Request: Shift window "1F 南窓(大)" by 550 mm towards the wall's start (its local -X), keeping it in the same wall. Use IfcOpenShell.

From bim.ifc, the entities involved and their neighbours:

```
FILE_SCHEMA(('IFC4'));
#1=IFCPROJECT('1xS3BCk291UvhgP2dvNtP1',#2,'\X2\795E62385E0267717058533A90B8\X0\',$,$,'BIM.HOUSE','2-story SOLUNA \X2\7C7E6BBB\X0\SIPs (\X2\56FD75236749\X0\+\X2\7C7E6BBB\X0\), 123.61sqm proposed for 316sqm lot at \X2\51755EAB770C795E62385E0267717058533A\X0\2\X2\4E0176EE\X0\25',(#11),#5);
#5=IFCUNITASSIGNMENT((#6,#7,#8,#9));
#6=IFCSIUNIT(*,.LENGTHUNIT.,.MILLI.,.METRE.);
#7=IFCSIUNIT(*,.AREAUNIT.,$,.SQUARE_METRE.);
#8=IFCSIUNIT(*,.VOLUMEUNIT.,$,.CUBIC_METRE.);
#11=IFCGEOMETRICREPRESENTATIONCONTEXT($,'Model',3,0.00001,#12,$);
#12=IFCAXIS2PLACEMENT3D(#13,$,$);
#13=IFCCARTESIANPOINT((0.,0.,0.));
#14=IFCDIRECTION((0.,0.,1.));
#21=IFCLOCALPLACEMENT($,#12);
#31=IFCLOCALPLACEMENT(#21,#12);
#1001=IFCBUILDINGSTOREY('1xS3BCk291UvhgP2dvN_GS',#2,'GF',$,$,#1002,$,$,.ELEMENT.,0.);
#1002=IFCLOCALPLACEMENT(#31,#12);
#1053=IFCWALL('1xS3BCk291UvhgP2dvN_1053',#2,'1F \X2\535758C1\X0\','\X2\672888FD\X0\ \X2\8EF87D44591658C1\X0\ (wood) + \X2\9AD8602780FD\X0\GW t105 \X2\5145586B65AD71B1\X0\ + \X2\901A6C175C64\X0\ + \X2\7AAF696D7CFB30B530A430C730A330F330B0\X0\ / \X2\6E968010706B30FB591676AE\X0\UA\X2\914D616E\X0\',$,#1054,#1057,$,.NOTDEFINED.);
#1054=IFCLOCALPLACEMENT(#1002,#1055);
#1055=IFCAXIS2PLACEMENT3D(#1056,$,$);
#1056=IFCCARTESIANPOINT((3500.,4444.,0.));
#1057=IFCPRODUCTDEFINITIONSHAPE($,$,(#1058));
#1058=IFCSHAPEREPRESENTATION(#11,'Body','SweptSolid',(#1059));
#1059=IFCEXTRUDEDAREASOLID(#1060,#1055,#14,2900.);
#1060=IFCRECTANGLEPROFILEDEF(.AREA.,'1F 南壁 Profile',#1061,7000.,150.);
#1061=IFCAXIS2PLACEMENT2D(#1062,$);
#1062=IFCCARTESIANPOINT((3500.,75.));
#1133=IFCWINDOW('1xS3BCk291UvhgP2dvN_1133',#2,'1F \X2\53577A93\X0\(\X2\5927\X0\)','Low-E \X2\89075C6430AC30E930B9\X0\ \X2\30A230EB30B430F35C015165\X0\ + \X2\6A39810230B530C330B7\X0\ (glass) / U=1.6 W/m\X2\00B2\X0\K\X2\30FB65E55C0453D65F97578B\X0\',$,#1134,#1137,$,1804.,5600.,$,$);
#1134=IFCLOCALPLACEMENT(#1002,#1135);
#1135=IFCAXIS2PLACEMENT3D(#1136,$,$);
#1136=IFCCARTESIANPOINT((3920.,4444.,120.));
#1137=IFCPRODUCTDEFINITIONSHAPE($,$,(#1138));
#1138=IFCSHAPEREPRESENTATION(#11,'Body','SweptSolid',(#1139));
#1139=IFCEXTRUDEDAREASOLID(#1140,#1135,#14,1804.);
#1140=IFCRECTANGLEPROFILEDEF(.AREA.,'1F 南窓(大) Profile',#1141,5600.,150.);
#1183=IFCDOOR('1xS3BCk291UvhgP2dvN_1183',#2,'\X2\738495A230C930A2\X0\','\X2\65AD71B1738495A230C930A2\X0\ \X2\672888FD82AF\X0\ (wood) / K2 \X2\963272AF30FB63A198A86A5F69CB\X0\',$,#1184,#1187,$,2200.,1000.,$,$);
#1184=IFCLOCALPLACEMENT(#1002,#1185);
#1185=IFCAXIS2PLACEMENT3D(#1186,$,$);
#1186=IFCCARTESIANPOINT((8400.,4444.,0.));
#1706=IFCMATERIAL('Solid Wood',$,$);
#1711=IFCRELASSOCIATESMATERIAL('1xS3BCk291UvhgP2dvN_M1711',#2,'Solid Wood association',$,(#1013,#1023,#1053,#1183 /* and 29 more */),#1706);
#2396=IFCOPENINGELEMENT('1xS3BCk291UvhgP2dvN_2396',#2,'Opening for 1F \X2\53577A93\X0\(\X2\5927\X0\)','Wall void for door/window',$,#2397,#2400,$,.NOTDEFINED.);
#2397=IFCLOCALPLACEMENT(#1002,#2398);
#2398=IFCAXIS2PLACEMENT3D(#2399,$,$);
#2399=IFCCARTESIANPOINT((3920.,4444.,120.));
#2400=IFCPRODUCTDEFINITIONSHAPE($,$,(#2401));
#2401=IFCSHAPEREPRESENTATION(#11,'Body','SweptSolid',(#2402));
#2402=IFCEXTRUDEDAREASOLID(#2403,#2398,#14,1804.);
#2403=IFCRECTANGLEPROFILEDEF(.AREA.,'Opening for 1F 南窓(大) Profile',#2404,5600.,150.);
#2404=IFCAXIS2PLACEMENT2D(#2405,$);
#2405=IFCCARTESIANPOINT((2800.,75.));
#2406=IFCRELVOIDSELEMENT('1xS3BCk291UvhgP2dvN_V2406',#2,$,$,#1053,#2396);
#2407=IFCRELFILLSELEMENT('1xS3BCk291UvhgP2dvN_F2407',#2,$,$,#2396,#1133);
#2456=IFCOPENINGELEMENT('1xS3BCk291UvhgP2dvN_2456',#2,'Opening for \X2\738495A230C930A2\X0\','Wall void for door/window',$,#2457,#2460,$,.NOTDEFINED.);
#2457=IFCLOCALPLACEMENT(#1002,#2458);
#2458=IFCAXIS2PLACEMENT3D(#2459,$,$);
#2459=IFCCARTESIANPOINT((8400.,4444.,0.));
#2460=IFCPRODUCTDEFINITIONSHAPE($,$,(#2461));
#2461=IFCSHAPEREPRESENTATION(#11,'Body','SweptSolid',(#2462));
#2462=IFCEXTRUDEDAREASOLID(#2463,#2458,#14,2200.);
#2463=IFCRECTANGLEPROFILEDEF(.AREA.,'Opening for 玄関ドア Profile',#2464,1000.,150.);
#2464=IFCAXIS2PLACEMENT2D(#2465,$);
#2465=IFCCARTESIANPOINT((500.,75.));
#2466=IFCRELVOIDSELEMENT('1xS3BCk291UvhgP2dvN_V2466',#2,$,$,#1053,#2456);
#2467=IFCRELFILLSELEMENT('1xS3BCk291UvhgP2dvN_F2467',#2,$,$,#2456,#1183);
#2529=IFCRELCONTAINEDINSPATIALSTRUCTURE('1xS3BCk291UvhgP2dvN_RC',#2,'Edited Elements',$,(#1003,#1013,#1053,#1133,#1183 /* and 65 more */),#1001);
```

```python
import ifcopenshell
import ifcopenshell.api.geometry
import ifcopenshell.util.placement
import ifcopenshell.util.unit

model = ifcopenshell.open("bim.ifc")
unit_scale = ifcopenshell.util.unit.calculate_unit_scale(model)

window = model.by_id(1133)
opening = window.FillsVoids[0].RelatingOpeningElement
wall = opening.VoidsElements[0].RelatingBuildingElement

wall_matrix = ifcopenshell.util.placement.get_local_placement(wall.ObjectPlacement)
shift = wall_matrix[:3, 0] * -0.55 / unit_scale
before = ifcopenshell.util.placement.get_local_placement(window.ObjectPlacement)[:3, 3].copy()

# The window is not placed relative to its opening, so move both.
for product in (opening, window):
    matrix = ifcopenshell.util.placement.get_local_placement(product.ObjectPlacement)
    matrix[:3, 3] += shift
    ifcopenshell.api.geometry.edit_object_placement(model, product=product, matrix=matrix, is_si=False)

after = ifcopenshell.util.placement.get_local_placement(window.ObjectPlacement)[:3, 3]
print("window moved by", (after - before).round(3) + 0.0)

model.write("bim_updated.ifc")
```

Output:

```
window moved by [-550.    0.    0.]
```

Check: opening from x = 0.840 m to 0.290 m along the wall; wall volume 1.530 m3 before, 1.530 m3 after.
